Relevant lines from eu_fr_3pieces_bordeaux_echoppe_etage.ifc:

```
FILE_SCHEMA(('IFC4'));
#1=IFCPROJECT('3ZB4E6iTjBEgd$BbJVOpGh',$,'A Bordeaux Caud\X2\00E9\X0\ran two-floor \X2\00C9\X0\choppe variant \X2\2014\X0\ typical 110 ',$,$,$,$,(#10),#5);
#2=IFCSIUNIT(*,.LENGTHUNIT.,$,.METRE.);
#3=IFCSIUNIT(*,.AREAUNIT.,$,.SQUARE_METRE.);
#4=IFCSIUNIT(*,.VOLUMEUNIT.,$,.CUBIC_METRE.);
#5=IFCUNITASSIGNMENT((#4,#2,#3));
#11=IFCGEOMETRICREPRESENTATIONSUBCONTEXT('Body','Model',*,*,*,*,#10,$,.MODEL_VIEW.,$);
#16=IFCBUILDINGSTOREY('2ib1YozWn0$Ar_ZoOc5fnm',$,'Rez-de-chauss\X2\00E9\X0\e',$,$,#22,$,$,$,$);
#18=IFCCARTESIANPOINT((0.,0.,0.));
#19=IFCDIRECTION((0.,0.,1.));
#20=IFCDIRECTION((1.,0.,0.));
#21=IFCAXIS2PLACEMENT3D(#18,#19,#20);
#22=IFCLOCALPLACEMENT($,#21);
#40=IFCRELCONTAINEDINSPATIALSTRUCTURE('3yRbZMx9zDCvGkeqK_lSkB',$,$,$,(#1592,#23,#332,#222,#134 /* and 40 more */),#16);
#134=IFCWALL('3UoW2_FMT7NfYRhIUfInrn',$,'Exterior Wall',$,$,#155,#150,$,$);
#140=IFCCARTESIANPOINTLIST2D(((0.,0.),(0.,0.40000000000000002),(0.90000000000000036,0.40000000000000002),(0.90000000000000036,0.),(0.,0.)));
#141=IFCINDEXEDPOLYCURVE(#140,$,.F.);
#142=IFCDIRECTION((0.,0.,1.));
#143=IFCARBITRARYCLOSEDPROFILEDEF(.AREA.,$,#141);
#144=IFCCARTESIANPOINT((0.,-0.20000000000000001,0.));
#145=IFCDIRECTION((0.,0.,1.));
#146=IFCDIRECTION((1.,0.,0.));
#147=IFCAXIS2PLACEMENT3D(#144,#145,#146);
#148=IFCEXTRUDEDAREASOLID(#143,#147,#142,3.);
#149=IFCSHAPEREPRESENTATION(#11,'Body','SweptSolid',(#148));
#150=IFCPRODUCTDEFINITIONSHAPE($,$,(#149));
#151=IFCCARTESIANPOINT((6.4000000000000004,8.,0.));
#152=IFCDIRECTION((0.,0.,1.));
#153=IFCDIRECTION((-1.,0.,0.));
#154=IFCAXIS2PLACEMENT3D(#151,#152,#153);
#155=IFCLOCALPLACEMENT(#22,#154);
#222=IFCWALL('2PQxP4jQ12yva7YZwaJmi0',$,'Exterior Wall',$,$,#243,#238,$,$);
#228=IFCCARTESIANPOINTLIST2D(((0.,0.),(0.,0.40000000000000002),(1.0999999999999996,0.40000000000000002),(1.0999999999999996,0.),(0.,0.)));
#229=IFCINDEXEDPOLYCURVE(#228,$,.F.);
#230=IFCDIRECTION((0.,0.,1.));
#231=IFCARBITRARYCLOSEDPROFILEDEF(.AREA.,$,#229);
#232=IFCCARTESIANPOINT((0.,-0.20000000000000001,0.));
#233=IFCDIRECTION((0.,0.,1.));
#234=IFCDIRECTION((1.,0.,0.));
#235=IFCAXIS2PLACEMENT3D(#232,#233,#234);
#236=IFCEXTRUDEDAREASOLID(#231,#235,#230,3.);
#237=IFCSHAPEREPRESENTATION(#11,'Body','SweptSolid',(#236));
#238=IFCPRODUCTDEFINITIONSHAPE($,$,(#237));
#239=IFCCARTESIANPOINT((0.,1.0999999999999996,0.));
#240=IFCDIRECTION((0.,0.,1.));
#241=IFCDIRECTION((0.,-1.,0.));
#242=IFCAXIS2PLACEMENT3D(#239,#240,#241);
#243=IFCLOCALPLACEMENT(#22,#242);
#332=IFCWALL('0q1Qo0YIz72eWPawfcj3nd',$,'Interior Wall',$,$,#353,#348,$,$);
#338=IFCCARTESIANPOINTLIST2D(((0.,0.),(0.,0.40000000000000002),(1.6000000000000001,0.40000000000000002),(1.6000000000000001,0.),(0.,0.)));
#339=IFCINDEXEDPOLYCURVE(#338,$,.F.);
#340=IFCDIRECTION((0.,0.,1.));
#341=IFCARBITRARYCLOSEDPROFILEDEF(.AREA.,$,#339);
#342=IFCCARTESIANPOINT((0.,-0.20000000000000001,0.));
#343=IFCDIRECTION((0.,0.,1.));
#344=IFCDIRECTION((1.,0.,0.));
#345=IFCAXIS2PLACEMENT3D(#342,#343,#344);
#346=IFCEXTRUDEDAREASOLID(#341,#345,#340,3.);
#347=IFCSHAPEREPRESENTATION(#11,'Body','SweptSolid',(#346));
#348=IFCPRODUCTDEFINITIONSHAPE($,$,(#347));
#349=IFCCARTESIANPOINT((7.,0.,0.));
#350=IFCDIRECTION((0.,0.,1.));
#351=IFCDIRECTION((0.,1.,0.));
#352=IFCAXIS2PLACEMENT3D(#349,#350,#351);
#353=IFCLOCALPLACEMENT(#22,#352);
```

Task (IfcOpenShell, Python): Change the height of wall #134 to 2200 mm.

```python
import ifcopenshell
import ifcopenshell.geom
import ifcopenshell.util.representation
import ifcopenshell.util.shape
import ifcopenshell.util.unit

model = ifcopenshell.open("eu_fr_3pieces_bordeaux_echoppe_etage.ifc")
unit_scale = ifcopenshell.util.unit.calculate_unit_scale(model)
settings = ifcopenshell.geom.settings()


def volume(element):
    """Net volume in cubic metres, openings subtracted."""
    shape = ifcopenshell.geom.create_shape(settings, element)
    return ifcopenshell.util.shape.get_volume(shape.geometry)


wall = model.by_guid("3UoW2_FMT7NfYRhIUfInrn")
before = volume(wall)

body = ifcopenshell.util.representation.get_representation(wall, "Model", "Body")
solid = body.Items[0]
old_height = solid.Depth
solid.Depth = 2.2 / unit_scale
after = volume(wall)

print(f"height {old_height:g} -> {solid.Depth:g}, volume {before:.3f} -> {after:.3f} m3")

model.write("eu_fr_3pieces_bordeaux_echoppe_etage-out.ifc")
```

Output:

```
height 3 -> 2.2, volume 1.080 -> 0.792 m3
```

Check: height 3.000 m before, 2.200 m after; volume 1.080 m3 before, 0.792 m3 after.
